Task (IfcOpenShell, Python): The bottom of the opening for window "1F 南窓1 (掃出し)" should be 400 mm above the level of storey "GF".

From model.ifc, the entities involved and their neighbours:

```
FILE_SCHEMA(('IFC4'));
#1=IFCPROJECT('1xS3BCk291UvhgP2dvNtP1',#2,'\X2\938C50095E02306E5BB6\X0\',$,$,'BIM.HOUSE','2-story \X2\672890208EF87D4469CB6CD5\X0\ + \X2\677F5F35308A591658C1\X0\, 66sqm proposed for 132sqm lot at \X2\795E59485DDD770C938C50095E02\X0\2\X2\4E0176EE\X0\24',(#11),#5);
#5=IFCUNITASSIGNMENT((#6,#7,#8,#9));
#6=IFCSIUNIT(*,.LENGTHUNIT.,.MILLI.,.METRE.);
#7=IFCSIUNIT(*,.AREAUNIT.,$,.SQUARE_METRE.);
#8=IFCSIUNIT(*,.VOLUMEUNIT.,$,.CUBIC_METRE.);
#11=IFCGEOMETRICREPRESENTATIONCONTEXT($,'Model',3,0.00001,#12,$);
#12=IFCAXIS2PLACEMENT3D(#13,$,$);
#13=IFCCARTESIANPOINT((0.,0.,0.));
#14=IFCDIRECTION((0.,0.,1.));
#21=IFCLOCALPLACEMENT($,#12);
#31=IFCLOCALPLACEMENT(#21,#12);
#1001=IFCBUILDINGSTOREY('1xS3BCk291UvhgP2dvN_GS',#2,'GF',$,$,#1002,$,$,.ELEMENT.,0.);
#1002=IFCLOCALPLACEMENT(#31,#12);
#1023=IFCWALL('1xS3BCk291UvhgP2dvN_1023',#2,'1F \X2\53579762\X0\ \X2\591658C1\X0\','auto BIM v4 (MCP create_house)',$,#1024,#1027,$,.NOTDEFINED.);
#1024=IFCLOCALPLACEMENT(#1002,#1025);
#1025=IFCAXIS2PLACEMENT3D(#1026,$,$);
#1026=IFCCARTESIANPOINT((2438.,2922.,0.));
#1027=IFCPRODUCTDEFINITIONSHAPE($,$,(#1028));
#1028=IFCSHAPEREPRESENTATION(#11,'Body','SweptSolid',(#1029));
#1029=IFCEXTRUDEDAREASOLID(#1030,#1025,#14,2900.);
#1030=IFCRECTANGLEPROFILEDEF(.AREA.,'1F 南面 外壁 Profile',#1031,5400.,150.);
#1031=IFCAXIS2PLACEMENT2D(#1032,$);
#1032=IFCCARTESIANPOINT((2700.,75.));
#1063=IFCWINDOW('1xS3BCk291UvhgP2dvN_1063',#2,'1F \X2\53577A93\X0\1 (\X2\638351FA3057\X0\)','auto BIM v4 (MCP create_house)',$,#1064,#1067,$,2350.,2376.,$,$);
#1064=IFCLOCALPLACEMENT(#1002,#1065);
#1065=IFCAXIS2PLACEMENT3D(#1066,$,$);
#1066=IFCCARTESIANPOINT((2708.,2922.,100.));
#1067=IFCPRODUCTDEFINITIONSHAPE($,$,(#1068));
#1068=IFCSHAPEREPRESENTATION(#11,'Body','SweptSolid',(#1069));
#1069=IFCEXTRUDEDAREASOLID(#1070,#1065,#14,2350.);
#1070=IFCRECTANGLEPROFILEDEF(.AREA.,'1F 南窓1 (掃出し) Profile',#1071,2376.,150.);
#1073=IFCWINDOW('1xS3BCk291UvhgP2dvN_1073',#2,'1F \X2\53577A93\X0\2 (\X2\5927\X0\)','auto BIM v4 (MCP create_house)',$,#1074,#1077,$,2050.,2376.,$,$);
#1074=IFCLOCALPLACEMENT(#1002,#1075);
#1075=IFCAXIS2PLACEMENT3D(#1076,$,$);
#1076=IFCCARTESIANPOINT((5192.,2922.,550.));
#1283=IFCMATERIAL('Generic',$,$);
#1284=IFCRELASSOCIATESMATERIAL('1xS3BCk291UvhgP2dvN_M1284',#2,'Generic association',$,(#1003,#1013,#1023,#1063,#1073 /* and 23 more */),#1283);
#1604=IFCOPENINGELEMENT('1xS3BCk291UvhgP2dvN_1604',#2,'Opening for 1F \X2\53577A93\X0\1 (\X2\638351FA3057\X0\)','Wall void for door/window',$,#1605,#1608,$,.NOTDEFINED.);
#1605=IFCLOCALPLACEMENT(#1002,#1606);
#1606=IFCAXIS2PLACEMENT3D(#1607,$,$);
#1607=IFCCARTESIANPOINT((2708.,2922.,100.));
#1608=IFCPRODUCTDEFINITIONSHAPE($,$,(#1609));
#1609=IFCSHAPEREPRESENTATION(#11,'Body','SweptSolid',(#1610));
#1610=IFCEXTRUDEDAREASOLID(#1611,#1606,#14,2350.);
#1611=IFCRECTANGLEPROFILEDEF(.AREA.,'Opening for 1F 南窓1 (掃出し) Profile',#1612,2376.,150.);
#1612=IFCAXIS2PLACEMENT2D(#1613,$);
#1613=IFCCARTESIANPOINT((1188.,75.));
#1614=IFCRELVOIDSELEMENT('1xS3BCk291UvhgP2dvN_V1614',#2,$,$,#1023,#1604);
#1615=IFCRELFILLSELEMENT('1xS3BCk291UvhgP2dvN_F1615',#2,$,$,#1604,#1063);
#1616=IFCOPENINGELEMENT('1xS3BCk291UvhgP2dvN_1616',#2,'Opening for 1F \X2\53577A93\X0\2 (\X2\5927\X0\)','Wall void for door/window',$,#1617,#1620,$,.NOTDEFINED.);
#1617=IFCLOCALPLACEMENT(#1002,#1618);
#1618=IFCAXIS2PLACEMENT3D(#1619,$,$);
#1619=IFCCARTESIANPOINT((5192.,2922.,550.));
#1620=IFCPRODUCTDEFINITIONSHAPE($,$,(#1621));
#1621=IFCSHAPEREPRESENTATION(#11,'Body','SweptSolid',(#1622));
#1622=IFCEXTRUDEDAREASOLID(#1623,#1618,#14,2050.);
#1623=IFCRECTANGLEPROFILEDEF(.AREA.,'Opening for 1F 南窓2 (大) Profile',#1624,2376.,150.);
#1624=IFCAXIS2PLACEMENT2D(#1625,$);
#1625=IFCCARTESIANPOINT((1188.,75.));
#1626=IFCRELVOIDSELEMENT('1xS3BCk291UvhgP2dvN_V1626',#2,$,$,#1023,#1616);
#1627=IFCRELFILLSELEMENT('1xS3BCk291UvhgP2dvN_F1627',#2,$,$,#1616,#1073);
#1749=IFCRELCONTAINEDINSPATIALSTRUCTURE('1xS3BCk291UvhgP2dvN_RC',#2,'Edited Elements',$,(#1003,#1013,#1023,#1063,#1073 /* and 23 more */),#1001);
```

```python
import numpy as np
import ifcopenshell
import ifcopenshell.api.geometry
import ifcopenshell.geom
import ifcopenshell.util.element
import ifcopenshell.util.placement
import ifcopenshell.util.shape
import ifcopenshell.util.unit

model = ifcopenshell.open("model.ifc")
unit_scale = ifcopenshell.util.unit.calculate_unit_scale(model)

window = model.by_guid("1xS3BCk291UvhgP2dvN_1063")
opening = window.FillsVoids[0].RelatingOpeningElement
storey = ifcopenshell.util.element.get_container(window, ifc_class="IfcBuildingStorey")
level = ifcopenshell.util.placement.get_local_placement(storey.ObjectPlacement)[2, 3]

# The opening's origin need not be at the sill, so measure its lowest point.
shape = ifcopenshell.geom.create_shape(ifcopenshell.geom.settings(), opening)
bottom = ifcopenshell.util.shape.get_shape_bottom_elevation(shape, shape.geometry) / unit_scale
dz = level + 0.4 / unit_scale - bottom

shift = np.array([0.0, 0.0, dz])
# The window is not placed relative to its opening, so move both.
for product in (opening, window):
    matrix = ifcopenshell.util.placement.get_local_placement(product.ObjectPlacement)
    matrix[:3, 3] += shift
    ifcopenshell.api.geometry.edit_object_placement(model, product=product, matrix=matrix, is_si=False)

print(f"moved by {dz * unit_scale:+.3f} m")

model.write("model-out.ifc")
```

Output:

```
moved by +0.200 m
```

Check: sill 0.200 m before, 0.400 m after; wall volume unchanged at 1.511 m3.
